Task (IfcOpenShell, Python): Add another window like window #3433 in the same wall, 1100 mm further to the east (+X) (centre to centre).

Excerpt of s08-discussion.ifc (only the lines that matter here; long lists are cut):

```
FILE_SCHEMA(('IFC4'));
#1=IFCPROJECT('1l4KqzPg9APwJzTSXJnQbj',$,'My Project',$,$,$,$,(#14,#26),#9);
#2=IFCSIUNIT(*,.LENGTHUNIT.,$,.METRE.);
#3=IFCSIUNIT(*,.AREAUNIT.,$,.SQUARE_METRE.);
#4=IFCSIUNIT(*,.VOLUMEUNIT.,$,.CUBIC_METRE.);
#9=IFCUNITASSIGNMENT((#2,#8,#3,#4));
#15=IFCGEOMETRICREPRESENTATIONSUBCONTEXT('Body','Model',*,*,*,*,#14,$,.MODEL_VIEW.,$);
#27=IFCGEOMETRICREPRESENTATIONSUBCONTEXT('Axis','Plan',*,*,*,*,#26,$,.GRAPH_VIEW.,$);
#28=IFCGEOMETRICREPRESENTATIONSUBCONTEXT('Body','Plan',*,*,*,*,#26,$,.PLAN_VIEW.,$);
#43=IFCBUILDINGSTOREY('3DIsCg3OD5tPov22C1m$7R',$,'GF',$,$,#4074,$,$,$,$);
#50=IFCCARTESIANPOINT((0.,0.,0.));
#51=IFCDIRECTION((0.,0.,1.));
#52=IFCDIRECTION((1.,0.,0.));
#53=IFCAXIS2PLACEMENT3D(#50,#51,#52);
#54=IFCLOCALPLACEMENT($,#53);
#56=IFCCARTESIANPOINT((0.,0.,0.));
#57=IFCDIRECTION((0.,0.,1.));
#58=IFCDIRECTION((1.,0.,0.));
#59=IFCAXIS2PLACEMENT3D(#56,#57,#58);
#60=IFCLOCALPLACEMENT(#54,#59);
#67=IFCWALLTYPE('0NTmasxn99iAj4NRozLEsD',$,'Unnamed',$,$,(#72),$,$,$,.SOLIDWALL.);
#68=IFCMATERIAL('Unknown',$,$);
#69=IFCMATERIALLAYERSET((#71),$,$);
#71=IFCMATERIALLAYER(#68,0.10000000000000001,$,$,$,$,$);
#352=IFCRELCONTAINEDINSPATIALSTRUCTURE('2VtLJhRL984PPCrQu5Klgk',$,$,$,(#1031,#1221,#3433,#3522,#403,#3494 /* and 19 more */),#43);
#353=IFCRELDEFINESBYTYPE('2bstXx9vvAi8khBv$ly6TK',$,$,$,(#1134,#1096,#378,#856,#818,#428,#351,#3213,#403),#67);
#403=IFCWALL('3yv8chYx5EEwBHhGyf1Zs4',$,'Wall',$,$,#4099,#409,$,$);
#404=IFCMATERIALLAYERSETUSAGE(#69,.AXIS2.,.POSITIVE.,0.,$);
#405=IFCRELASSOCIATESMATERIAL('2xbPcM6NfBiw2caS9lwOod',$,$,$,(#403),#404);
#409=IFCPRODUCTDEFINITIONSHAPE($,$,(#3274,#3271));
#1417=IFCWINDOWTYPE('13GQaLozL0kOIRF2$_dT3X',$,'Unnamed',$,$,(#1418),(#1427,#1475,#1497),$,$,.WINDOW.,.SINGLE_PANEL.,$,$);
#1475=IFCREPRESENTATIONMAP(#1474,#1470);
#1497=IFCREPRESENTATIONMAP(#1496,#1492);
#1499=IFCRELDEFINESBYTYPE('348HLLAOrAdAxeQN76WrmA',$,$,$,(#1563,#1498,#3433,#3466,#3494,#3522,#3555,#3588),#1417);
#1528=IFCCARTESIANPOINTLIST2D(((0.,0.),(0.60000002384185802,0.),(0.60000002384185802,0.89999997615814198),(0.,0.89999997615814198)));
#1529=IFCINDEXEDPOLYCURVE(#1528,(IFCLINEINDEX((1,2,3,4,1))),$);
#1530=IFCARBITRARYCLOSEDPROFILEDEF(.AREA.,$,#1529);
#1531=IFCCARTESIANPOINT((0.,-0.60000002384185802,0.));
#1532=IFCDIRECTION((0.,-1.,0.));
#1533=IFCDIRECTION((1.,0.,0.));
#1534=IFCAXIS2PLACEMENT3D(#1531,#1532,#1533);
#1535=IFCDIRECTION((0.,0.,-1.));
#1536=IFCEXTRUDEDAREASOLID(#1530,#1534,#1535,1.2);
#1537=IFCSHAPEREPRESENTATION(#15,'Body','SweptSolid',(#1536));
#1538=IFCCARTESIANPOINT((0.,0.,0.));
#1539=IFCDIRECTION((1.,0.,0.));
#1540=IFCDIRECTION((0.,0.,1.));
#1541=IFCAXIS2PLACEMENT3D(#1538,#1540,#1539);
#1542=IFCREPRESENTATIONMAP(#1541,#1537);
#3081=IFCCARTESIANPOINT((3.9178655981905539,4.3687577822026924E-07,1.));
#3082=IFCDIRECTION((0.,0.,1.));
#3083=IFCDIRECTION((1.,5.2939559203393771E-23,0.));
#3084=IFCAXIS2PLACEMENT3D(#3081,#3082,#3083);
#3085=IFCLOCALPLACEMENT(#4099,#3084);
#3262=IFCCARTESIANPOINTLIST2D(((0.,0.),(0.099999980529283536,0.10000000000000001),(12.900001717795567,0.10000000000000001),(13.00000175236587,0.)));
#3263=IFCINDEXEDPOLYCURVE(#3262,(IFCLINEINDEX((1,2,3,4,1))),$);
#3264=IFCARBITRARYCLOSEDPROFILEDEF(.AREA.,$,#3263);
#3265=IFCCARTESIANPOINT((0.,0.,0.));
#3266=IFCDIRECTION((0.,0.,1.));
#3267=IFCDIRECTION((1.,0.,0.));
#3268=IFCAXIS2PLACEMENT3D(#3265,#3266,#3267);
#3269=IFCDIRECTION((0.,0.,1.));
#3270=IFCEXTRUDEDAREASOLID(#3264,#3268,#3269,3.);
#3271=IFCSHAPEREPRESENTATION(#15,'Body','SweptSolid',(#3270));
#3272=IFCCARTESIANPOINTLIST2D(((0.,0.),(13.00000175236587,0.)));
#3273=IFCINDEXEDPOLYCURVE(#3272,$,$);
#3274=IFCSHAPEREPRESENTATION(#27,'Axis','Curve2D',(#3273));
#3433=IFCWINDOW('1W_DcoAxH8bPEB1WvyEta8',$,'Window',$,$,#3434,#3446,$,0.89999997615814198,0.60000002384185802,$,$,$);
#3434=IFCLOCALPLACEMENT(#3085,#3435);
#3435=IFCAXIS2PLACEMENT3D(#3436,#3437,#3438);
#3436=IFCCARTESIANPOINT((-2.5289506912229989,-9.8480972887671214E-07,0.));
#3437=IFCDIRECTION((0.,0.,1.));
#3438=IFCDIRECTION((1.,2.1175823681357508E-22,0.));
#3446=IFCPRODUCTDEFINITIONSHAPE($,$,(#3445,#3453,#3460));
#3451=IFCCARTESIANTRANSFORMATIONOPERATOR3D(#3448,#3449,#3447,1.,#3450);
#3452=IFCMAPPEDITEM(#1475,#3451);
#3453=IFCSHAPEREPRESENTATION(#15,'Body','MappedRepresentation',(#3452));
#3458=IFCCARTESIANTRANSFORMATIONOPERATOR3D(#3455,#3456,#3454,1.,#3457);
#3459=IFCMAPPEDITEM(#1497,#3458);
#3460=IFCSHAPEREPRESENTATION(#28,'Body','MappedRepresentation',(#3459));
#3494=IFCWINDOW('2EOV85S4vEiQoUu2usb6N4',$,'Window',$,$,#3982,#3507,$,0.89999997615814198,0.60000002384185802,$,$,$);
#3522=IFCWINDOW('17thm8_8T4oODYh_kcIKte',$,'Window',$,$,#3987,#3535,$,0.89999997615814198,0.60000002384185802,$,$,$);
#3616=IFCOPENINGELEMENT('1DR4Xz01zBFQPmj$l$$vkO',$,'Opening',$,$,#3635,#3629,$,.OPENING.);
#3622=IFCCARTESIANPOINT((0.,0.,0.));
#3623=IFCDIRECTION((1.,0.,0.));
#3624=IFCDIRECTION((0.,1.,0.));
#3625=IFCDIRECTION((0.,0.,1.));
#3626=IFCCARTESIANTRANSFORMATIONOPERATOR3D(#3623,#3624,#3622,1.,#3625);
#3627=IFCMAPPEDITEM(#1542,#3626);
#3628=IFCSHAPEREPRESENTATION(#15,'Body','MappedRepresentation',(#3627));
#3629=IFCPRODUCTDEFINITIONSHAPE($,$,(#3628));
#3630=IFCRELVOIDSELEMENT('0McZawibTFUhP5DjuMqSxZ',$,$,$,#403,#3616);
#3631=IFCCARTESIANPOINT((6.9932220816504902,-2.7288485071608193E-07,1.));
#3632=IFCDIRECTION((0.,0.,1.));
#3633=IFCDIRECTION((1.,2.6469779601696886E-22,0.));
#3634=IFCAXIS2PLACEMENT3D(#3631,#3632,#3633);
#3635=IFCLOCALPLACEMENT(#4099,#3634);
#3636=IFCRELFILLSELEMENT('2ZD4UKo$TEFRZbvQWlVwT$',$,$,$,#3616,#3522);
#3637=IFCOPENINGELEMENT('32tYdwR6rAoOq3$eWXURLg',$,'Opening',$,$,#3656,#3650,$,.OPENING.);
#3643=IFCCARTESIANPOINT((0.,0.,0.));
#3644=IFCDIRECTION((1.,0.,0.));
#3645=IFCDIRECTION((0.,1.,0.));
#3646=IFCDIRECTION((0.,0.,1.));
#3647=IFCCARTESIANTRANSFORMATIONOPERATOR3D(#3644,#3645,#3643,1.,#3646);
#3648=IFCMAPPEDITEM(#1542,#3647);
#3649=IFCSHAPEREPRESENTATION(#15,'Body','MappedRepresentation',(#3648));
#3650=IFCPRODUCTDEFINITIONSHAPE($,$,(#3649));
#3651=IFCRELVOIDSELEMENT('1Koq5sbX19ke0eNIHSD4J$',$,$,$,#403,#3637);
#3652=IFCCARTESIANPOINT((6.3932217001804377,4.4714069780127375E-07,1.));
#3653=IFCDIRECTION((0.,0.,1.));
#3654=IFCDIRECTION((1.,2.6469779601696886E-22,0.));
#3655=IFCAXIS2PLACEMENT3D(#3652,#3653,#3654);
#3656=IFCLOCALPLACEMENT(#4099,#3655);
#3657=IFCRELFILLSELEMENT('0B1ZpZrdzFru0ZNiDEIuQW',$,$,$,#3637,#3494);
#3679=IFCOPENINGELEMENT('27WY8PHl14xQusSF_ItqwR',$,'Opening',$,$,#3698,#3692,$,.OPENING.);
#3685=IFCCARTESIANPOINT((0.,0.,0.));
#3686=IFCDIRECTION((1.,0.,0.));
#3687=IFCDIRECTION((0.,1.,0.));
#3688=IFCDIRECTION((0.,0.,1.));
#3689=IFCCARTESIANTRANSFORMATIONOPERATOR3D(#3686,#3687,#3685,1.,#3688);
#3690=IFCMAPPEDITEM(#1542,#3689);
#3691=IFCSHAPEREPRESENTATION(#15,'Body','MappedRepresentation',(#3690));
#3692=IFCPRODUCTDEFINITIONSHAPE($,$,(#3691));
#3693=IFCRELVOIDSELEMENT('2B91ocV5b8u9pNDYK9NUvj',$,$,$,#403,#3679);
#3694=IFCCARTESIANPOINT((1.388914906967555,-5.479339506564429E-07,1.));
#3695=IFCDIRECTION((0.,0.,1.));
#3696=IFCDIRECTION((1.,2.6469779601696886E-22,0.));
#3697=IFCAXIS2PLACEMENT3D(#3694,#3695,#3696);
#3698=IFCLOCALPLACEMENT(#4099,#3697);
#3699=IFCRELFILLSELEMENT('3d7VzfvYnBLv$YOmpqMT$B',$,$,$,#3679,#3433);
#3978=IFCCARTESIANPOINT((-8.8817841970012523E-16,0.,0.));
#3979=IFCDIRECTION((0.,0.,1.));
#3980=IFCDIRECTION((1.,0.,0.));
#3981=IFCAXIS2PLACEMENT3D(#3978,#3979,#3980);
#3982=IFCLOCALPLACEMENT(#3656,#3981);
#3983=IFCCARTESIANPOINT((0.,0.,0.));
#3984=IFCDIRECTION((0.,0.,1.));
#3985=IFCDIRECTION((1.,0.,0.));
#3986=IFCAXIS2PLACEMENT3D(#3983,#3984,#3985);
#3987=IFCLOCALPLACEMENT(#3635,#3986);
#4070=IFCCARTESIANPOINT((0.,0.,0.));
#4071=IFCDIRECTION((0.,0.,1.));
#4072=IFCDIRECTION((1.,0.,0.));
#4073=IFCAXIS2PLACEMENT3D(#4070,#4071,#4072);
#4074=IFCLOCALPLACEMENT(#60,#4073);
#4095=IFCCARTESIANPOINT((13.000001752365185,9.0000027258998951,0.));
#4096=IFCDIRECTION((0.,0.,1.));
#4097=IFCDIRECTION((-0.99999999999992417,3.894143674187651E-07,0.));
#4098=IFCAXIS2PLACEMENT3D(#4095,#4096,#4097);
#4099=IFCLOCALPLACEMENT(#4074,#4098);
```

```python
import ifcopenshell
import ifcopenshell.api.feature
import ifcopenshell.api.geometry
import ifcopenshell.api.root
import ifcopenshell.geom
import ifcopenshell.util.element
import ifcopenshell.util.placement
import ifcopenshell.util.shape

model = ifcopenshell.open("s08-discussion.ifc")
settings = ifcopenshell.geom.settings()


def volume(element):
    """Net volume in cubic metres, openings subtracted."""
    shape = ifcopenshell.geom.create_shape(settings, element)
    return ifcopenshell.util.shape.get_volume(shape.geometry)


window = model.by_guid("1W_DcoAxH8bPEB1WvyEta8")
opening = window.FillsVoids[0].RelatingOpeningElement
wall = opening.VoidsElements[0].RelatingBuildingElement
before = volume(wall)
shift = ifcopenshell.util.placement.get_local_placement(wall.ObjectPlacement)[:3, 0] * -1.1

# copy_class copies the void relationship, type, container and properties, but no geometry.
new_opening = ifcopenshell.api.root.copy_class(model, product=opening)
new_opening.Representation = ifcopenshell.util.element.copy_deep(
    model, opening.Representation, exclude=["IfcGeometricRepresentationContext", "IfcRepresentationMap"]
)
new_window = ifcopenshell.api.root.copy_class(model, product=window)
new_window.Representation = ifcopenshell.util.element.copy_deep(
    model, window.Representation, exclude=["IfcGeometricRepresentationContext", "IfcRepresentationMap"]
)
ifcopenshell.api.feature.add_filling(model, opening=new_opening, element=new_window)

for old, new in ((opening, new_opening), (window, new_window)):
    matrix = ifcopenshell.util.placement.get_local_placement(old.ObjectPlacement)
    matrix[:3, 3] += shift
    ifcopenshell.api.geometry.edit_object_placement(model, product=new, matrix=matrix, is_si=False)

after = volume(wall)

print(f"wall volume {before:.3f} -> {after:.3f} m3")

model.write("s08-discussion_rev.ifc")
```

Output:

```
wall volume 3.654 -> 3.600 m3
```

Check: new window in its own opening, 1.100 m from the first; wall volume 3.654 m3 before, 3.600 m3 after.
